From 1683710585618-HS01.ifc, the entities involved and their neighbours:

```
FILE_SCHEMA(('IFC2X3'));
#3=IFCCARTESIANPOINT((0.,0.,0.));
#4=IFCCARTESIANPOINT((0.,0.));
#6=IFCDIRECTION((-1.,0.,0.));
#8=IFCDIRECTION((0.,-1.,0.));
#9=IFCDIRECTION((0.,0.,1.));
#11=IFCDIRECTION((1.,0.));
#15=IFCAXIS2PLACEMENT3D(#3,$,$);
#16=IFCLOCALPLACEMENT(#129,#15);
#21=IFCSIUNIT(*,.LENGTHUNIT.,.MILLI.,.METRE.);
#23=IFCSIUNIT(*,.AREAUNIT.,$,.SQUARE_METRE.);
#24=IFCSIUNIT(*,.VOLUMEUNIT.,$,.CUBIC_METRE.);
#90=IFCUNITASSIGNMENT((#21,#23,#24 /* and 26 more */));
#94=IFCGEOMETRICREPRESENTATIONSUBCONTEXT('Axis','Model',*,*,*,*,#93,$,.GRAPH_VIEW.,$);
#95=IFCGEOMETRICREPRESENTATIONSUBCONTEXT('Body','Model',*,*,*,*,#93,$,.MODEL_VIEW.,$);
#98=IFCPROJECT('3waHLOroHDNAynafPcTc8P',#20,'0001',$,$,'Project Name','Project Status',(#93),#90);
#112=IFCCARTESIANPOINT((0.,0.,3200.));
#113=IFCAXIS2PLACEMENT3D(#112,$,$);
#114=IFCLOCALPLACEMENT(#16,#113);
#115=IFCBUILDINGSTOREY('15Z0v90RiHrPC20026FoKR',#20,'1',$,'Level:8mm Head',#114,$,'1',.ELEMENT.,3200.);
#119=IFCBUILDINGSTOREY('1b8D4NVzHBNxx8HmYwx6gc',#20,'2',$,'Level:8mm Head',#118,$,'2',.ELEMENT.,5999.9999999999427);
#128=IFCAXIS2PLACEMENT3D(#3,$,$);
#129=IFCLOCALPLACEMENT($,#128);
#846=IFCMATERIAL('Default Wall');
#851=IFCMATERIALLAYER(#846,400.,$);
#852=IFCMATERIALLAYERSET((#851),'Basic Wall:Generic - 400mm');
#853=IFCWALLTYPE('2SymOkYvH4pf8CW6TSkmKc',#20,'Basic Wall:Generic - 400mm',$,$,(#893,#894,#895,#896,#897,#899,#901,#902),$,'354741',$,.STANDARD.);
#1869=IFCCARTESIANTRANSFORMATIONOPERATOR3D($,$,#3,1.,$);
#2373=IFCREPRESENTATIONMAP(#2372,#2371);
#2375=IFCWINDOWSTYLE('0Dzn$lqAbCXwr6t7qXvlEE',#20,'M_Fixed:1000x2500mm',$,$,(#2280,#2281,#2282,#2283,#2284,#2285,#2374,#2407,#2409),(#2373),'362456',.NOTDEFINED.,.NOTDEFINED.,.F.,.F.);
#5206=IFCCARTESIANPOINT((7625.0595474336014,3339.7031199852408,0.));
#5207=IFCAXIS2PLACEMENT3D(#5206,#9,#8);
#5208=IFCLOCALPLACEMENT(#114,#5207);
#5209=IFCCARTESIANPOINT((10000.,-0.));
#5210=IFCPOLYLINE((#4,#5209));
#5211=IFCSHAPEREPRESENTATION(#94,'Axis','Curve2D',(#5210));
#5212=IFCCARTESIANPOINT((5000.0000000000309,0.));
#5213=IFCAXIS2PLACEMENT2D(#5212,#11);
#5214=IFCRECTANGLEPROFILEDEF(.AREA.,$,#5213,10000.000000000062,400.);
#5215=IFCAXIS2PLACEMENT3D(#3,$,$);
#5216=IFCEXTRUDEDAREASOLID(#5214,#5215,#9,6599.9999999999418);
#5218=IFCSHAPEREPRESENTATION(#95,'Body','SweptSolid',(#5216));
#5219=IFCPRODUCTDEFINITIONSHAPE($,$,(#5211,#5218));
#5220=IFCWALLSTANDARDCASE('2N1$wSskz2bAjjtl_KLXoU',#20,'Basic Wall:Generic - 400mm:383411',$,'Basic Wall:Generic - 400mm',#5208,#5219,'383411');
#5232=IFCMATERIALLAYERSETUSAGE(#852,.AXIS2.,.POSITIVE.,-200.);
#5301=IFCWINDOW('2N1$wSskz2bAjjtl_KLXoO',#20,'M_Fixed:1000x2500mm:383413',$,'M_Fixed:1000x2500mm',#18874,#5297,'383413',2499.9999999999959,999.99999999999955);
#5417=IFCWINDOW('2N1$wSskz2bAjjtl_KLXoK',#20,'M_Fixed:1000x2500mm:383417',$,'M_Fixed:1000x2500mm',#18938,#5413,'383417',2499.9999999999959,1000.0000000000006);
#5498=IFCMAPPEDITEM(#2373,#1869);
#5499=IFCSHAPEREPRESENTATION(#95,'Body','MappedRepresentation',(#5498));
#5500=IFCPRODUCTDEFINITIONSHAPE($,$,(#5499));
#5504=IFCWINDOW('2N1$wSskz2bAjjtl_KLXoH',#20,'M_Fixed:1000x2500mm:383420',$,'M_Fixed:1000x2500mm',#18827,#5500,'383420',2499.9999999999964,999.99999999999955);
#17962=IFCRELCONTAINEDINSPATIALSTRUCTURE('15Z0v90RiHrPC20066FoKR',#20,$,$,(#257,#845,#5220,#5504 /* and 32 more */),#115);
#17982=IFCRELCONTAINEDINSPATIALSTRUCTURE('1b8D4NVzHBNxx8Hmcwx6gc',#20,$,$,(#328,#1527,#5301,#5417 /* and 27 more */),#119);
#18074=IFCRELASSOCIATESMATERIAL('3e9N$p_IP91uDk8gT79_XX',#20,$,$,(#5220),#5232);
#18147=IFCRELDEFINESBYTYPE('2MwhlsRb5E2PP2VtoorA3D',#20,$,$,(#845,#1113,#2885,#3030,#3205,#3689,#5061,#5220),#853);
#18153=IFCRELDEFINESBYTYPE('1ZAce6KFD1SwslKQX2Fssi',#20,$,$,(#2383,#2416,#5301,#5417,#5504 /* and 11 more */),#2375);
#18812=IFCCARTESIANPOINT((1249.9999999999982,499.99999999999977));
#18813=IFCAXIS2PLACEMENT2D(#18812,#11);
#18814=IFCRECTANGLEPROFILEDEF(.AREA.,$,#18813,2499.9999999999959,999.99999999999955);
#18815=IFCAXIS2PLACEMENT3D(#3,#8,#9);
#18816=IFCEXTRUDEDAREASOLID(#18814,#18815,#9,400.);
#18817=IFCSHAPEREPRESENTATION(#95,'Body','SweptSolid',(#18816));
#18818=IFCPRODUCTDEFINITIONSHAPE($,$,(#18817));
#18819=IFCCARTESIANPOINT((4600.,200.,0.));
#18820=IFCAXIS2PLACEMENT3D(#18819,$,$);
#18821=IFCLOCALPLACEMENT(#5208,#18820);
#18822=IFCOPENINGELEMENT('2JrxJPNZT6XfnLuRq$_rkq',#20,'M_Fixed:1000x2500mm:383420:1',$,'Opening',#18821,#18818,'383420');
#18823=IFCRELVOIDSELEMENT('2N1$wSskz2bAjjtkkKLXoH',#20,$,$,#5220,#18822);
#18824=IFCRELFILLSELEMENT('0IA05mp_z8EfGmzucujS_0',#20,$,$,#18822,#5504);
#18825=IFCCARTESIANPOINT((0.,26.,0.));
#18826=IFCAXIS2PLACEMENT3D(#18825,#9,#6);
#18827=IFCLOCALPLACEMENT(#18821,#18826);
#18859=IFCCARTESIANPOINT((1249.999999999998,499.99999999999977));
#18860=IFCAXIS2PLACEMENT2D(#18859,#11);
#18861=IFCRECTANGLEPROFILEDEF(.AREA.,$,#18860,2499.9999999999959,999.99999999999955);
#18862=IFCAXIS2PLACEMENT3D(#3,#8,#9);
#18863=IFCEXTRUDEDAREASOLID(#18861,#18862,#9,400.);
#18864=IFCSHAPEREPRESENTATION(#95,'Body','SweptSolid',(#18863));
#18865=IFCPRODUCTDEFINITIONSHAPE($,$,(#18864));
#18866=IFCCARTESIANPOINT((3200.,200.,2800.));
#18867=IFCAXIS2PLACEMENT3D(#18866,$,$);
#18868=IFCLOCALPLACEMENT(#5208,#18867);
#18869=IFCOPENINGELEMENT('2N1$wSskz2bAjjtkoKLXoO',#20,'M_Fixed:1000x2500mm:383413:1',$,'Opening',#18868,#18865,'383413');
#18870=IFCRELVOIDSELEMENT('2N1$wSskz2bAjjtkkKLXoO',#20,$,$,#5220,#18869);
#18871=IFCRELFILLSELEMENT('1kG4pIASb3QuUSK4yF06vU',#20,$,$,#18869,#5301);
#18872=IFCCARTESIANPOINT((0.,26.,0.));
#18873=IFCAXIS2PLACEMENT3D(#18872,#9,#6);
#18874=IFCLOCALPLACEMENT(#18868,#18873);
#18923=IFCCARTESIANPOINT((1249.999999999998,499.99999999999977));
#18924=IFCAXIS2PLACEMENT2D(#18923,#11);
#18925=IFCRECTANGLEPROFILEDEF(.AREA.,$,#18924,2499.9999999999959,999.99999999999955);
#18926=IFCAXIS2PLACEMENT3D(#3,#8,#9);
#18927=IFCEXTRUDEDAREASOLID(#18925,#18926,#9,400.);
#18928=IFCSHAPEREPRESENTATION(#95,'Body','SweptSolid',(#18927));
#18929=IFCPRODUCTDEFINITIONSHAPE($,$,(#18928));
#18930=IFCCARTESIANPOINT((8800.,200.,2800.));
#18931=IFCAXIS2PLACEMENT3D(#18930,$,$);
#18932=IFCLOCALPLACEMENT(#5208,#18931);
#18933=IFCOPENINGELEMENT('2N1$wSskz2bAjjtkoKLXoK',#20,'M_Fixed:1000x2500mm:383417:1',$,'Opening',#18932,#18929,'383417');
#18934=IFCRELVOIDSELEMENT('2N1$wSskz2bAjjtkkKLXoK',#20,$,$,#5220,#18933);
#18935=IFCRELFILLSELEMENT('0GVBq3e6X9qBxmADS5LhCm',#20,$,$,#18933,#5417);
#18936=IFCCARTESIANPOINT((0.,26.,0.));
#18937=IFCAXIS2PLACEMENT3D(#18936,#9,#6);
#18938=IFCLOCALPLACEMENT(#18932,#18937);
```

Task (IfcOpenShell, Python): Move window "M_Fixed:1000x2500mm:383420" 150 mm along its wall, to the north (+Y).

```python
import ifcopenshell
import ifcopenshell.api.geometry
import ifcopenshell.util.placement

model = ifcopenshell.open("1683710585618-HS01.ifc")

window = model.by_guid("2N1$wSskz2bAjjtl_KLXoH")
opening = window.FillsVoids[0].RelatingOpeningElement
wall = opening.VoidsElements[0].RelatingBuildingElement

wall_matrix = ifcopenshell.util.placement.get_local_placement(wall.ObjectPlacement)
shift = wall_matrix[:3, 0] * -150.0
before = ifcopenshell.util.placement.get_local_placement(window.ObjectPlacement)[:3, 3].copy()

# The window is placed relative to its opening, so it follows when the opening moves.
matrix = ifcopenshell.util.placement.get_local_placement(opening.ObjectPlacement)
matrix[:3, 3] += shift
ifcopenshell.api.geometry.edit_object_placement(
    model, product=opening, matrix=matrix, is_si=False, should_transform_children=True
)

after = ifcopenshell.util.placement.get_local_placement(window.ObjectPlacement)[:3, 3]
print("window moved by", (after - before).round(3) + 0.0)

model.write("1683710585618-HS01_rev.ifc")
```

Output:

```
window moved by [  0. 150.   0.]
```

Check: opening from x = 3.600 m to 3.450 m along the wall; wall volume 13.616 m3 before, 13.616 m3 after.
